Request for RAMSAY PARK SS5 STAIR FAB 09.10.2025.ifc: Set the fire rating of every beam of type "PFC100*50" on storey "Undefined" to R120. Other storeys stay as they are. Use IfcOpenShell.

First a look at what the model holds.

```python
import ifcopenshell
import ifcopenshell.util.element

model = ifcopenshell.open("RAMSAY PARK SS5 STAIR FAB 09.10.2025.ifc")
print(model.schema)
storey = next(s for s in model.by_type("IfcBuildingStorey") if s.Name == "Undefined")
beams = [e for e in ifcopenshell.util.element.get_decomposition(storey) if e.is_a("IfcBeam")]
seen = {}
for e in beams:
    element_type = ifcopenshell.util.element.get_type(e)
    key = (element_type.Name if element_type != e and element_type else None, ifcopenshell.util.element.get_pset(e, "Pset_BeamCommon", "FireRating"))
    seen[key] = seen.get(key, 0) + 1
for (name, value), count in sorted(seen.items(), key=str):
    print(count, "x", name, "|", value)
```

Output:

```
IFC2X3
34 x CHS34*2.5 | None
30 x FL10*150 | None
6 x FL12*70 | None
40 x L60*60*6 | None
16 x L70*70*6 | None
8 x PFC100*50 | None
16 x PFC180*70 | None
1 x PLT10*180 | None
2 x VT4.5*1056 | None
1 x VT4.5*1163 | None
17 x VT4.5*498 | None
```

```python
import ifcopenshell
import ifcopenshell.api.pset
import ifcopenshell.util.element

model = ifcopenshell.open("RAMSAY PARK SS5 STAIR FAB 09.10.2025.ifc")

storey = next(s for s in model.by_type("IfcBuildingStorey") if s.Name == "Undefined")
beams = [e for e in ifcopenshell.util.element.get_decomposition(storey) if e.is_a("IfcBeam")]

count = 0
for e in beams:
    element_type = ifcopenshell.util.element.get_type(e)
    if element_type in (None, e) or element_type.Name != "PFC100*50":
        continue
    found = ifcopenshell.util.element.get_pset(e, "Pset_BeamCommon", should_inherit=False)
    if found:
        pset = model.by_id(found["id"])
        if len(ifcopenshell.util.element.get_elements_by_pset(pset)) > 1:
            pset = ifcopenshell.api.pset.unshare_pset(model, products=[e], pset=pset)[0]
    else:
        pset = ifcopenshell.api.pset.add_pset(model, product=e, name="Pset_BeamCommon")
    ifcopenshell.api.pset.edit_pset(model, pset=pset, properties={"FireRating": "R120"})
    count += 1

print(count, "beams updated")

model.write("RAMSAY PARK SS5 STAIR FAB 09.10.2025_updated.ifc")
```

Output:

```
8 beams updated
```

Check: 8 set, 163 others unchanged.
